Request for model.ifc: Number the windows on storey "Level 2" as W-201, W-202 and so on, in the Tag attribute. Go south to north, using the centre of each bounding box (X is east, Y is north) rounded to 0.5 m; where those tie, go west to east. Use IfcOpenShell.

First a look at what the model holds.

```python
import ifcopenshell
import ifcopenshell.util.element
import ifcopenshell.util.placement

model = ifcopenshell.open("model.ifc")
print(model.schema)
storey = next(s for s in model.by_type("IfcBuildingStorey") if s.Name == "Level 2")
windows = [e for e in ifcopenshell.util.element.get_decomposition(storey) if e.is_a("IfcWindow")]
for e in sorted(windows, key=lambda e: e.id()):
    origin = ifcopenshell.util.placement.get_local_placement(e.ObjectPlacement)[:3, 3]
    print(e.id(), e.Tag, e.Name, origin.round(2) + 0.0, sep=" | ")
```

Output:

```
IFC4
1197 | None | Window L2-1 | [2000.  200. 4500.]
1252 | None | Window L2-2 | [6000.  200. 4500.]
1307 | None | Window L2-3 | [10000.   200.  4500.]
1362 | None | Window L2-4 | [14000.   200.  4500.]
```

```python
import ifcopenshell
import ifcopenshell.geom
import ifcopenshell.util.element
import ifcopenshell.util.shape

model = ifcopenshell.open("model.ifc")
settings = ifcopenshell.geom.settings()
settings.set("use-world-coords", True)


def centre(element):
    shape = ifcopenshell.geom.create_shape(settings, element)
    return ifcopenshell.util.shape.get_bbox_centroid(shape.geometry)


storey = next(s for s in model.by_type("IfcBuildingStorey") if s.Name == "Level 2")
windows = [e for e in ifcopenshell.util.element.get_decomposition(storey) if e.is_a("IfcWindow")]

# Insertion points can sit at a corner or the storey origin, so sort by the geometry (in metres).
centres = {e: centre(e) for e in windows}
windows.sort(key=lambda e: (round(centres[e][1] / 0.5), centres[e][0]))

for i, e in enumerate(windows, start=1):
    number = f"W-2{i:02d}"
    e.Tag = number
    print(e.id(), number)

model.write("model-out.ifc")
```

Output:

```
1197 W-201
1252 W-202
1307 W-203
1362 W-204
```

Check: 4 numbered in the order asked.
